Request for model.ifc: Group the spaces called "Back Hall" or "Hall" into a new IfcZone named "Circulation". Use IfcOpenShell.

First a look at what the model holds.

```python
import ifcopenshell

model = ifcopenshell.open("model.ifc")
print(model.schema)
seen = {}
for space in model.by_type("IfcSpace"):
    seen[space.LongName] = seen.get(space.LongName, 0) + 1
for name, count in sorted(seen.items(), key=str):
    print(count, "x", name)
print("zones:", [z.Name for z in model.by_type("IfcZone")][:20])
```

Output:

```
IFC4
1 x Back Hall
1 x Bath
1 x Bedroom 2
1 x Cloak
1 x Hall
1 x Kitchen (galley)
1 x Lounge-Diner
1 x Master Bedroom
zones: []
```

```python
import ifcopenshell
import ifcopenshell.api.group
import ifcopenshell.api.root

model = ifcopenshell.open("model.ifc")

names = {"Back Hall", "Hall"}
spaces = [s for s in model.by_type("IfcSpace") if s.LongName in names]

zone = ifcopenshell.api.root.create_entity(model, ifc_class="IfcZone", name="Circulation")
ifcopenshell.api.group.assign_group(model, products=spaces, group=zone)
print(len(spaces), "spaces in", zone.Name)

model.write("model_edited.ifc")
```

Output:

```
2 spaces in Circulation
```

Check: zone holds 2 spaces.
